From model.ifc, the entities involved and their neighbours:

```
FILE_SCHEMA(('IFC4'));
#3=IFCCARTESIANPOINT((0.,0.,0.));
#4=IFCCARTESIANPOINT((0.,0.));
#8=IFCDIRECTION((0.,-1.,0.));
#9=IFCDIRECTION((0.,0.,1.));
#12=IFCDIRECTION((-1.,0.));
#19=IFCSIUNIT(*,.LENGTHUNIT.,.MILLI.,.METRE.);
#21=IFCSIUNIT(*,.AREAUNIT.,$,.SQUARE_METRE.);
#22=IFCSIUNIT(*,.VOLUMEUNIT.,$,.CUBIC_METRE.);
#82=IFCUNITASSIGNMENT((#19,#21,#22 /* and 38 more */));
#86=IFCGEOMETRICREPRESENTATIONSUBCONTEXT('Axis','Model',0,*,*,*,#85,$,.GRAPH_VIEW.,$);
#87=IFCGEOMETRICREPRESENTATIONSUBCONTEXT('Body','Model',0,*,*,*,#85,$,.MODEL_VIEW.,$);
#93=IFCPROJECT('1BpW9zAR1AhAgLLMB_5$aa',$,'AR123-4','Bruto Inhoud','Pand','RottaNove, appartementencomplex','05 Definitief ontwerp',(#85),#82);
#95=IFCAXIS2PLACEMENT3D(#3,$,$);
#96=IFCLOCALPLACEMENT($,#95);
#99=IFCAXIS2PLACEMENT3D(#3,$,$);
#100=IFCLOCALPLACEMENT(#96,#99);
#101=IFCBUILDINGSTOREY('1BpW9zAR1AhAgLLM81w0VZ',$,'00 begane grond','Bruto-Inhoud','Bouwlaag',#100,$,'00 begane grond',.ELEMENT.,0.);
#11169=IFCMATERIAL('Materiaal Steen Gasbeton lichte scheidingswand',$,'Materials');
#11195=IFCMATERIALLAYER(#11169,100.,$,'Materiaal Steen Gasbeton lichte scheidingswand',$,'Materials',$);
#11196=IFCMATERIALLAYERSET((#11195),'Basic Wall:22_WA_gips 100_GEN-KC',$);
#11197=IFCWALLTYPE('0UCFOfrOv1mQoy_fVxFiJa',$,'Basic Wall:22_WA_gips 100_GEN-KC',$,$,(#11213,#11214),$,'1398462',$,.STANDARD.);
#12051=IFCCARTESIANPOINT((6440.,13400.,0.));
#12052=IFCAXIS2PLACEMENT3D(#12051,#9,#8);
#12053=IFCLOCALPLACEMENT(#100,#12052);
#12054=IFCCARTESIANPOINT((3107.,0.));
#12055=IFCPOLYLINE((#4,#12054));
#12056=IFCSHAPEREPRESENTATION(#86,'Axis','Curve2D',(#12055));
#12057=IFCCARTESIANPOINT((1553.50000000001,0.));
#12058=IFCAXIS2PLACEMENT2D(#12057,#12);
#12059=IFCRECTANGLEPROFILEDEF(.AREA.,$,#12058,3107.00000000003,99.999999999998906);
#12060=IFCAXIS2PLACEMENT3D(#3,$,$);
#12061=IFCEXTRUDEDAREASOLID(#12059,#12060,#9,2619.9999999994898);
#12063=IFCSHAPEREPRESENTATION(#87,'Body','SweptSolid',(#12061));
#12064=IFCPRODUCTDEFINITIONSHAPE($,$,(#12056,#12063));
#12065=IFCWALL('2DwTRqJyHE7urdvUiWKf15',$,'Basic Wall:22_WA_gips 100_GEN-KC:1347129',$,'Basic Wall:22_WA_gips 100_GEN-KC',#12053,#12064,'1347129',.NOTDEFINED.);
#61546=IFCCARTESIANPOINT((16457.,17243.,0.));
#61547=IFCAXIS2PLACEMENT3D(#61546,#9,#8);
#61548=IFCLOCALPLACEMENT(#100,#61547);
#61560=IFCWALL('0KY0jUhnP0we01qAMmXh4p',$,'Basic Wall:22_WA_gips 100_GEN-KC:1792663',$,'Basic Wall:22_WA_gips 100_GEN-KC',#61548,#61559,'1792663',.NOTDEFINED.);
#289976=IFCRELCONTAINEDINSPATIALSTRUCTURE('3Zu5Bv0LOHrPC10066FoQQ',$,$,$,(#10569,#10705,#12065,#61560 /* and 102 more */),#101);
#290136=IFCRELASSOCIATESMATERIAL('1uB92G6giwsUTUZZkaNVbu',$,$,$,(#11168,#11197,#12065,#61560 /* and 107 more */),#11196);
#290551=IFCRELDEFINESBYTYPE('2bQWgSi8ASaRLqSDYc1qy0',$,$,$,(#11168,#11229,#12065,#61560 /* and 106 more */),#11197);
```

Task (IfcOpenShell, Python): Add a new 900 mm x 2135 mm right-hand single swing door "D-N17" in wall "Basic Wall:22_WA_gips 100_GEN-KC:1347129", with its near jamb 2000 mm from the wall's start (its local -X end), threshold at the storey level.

```python
import numpy as np
import ifcopenshell
import ifcopenshell.api.feature
import ifcopenshell.api.geometry
import ifcopenshell.api.root
import ifcopenshell.api.spatial
import ifcopenshell.geom
import ifcopenshell.util.element
import ifcopenshell.util.placement
import ifcopenshell.util.representation
import ifcopenshell.util.shape
import ifcopenshell.util.unit

model = ifcopenshell.open("model.ifc")
unit_scale = ifcopenshell.util.unit.calculate_unit_scale(model)
settings = ifcopenshell.geom.settings()


def volume(element):
    """Net volume in cubic metres, openings subtracted."""
    shape = ifcopenshell.geom.create_shape(settings, element)
    return ifcopenshell.util.shape.get_volume(shape.geometry)


wall = model.by_guid("2DwTRqJyHE7urdvUiWKf15")
storey = ifcopenshell.util.element.get_container(wall, ifc_class="IfcBuildingStorey")
context = ifcopenshell.util.representation.get_context(model, "Model", "Body", "MODEL_VIEW")
before = volume(wall)

width, height, from_end, sill = 0.9, 2.135, 2, 0.0  # metres

# The wall runs along its own X axis, and the end named is its -X end.
wall_shape = ifcopenshell.geom.create_shape(settings, wall)
x, y, z = ifcopenshell.util.shape.get_vertices(wall_shape.geometry).T
start = x.min() + from_end
face, thickness = float(y.min()), float(y.max() - y.min())
wall_matrix = ifcopenshell.util.placement.get_local_placement(wall.ObjectPlacement)
level = ifcopenshell.util.placement.get_local_placement(storey.ObjectPlacement)[2, 3]


def in_wall(x, y):
    """Placement at x, y metres in the wall's axes, at sill height."""
    matrix = wall_matrix.copy()
    matrix[:, 3] = wall_matrix @ np.array([x / unit_scale, y / unit_scale, 0.0, 1.0])
    matrix[2, 3] = level + sill / unit_scale
    return matrix


# Opening: a box that overshoots both wall faces by 50 mm.
opening = ifcopenshell.api.root.create_entity(model, ifc_class="IfcOpeningElement", predefined_type="OPENING")
box = ifcopenshell.api.geometry.add_wall_representation(
    model, context=context, length=width, height=height, thickness=thickness + 0.1
)
ifcopenshell.api.geometry.assign_representation(model, product=opening, representation=box)
ifcopenshell.api.geometry.edit_object_placement(model, product=opening, matrix=in_wall(start, face - 0.05), is_si=False)
ifcopenshell.api.feature.add_feature(model, feature=opening, element=wall)

door = ifcopenshell.api.root.create_entity(model, ifc_class="IfcDoor", name="D-N17", predefined_type="DOOR")
door.OverallWidth, door.OverallHeight = width / unit_scale, height / unit_scale
door.OperationType = "SINGLE_SWING_RIGHT"
body = ifcopenshell.api.geometry.add_door_representation(
    model,
    context=context,
    overall_width=door.OverallWidth,
    overall_height=door.OverallHeight,
    operation_type="SINGLE_SWING_RIGHT",
    lining_properties={"LiningDepth": thickness / unit_scale, "ThresholdDepth": thickness / unit_scale},
)
ifcopenshell.api.geometry.assign_representation(model, product=door, representation=body)
ifcopenshell.api.spatial.assign_container(model, products=[door], relating_structure=storey)
ifcopenshell.api.feature.add_filling(model, opening=opening, element=door)

# The lining spans the wall, so the door starts at the wall face.
ifcopenshell.api.geometry.edit_object_placement(model, product=door, matrix=in_wall(start, face), is_si=False)

after = volume(wall)

print(f"wall volume {before:.3f} -> {after:.3f} m3")

model.write("model-out.ifc")
```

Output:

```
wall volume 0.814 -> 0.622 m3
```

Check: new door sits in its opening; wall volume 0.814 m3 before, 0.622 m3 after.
